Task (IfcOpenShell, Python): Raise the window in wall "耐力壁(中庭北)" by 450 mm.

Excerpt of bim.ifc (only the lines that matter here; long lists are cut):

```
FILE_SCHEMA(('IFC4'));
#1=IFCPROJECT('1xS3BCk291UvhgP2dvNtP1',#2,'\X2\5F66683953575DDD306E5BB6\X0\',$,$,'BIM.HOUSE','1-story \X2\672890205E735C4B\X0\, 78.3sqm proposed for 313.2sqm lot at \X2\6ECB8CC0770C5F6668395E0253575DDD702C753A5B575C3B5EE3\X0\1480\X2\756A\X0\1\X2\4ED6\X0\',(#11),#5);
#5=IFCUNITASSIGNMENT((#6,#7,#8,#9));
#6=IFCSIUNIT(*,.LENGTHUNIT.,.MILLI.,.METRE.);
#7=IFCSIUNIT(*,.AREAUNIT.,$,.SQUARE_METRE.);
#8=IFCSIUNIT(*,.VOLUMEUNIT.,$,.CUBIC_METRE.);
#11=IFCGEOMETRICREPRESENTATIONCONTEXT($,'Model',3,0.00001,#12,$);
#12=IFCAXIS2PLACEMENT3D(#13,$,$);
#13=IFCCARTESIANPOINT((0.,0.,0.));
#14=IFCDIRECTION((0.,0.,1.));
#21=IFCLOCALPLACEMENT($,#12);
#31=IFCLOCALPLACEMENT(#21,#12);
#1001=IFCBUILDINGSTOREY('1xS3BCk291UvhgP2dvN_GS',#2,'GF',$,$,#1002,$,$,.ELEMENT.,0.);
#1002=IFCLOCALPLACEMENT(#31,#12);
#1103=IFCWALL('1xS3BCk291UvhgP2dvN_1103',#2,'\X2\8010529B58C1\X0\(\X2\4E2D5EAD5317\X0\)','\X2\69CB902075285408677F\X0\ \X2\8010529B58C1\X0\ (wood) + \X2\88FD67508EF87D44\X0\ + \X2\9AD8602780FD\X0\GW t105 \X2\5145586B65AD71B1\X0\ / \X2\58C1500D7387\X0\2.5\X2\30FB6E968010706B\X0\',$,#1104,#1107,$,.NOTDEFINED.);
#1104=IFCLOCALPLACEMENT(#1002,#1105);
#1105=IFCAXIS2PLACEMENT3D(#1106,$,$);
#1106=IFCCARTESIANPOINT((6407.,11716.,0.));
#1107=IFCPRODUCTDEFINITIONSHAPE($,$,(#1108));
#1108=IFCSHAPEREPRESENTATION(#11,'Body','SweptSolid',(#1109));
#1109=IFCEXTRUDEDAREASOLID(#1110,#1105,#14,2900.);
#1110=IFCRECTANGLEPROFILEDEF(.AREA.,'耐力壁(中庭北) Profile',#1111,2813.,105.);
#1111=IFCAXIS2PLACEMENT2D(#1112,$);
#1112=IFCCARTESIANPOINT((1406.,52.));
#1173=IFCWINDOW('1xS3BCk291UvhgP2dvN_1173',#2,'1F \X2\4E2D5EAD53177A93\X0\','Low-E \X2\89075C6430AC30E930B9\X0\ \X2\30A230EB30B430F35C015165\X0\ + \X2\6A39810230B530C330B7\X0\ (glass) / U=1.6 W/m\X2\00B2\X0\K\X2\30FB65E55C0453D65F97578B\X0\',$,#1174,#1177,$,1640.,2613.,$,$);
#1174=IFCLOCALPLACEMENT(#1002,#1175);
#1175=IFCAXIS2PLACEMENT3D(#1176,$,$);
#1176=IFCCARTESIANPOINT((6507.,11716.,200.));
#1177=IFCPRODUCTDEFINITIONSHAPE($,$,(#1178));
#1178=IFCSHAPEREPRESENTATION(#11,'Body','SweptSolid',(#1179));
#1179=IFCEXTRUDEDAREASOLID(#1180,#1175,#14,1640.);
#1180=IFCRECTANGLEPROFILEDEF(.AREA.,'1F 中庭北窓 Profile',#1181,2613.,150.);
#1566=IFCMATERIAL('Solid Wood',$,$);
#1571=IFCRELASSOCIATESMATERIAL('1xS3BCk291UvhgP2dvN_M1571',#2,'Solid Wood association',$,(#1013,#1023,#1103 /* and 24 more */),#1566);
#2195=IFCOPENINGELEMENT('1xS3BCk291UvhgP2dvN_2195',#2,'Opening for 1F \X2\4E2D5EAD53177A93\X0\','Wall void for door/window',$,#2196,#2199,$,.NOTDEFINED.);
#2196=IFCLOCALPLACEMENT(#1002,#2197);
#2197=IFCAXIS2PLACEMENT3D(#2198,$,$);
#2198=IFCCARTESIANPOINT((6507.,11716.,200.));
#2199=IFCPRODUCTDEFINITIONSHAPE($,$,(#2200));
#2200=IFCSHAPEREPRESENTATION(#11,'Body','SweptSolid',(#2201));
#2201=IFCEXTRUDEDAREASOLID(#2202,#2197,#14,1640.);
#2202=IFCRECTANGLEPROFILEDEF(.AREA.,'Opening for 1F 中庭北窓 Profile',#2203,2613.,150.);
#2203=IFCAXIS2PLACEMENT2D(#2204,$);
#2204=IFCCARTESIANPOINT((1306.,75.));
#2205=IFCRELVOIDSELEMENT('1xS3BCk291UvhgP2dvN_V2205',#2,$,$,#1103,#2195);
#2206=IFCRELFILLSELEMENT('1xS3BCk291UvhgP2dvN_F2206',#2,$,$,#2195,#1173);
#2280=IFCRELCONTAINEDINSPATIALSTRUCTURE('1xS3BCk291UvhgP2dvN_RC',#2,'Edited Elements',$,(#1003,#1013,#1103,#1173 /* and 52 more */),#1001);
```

```python
import numpy as np
import ifcopenshell
import ifcopenshell.api.geometry
import ifcopenshell.util.placement
import ifcopenshell.util.unit

model = ifcopenshell.open("bim.ifc")
unit_scale = ifcopenshell.util.unit.calculate_unit_scale(model)

window = model.by_guid("1xS3BCk291UvhgP2dvN_1173")
opening = window.FillsVoids[0].RelatingOpeningElement
dz = 0.45 / unit_scale

shift = np.array([0.0, 0.0, dz])
# The window is not placed relative to its opening, so move both.
for product in (opening, window):
    matrix = ifcopenshell.util.placement.get_local_placement(product.ObjectPlacement)
    matrix[:3, 3] += shift
    ifcopenshell.api.geometry.edit_object_placement(model, product=product, matrix=matrix, is_si=False)

print(f"moved by {dz * unit_scale:+.3f} m")

model.write("bim_edited.ifc")
```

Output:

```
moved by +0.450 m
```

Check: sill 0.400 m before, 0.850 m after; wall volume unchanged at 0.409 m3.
